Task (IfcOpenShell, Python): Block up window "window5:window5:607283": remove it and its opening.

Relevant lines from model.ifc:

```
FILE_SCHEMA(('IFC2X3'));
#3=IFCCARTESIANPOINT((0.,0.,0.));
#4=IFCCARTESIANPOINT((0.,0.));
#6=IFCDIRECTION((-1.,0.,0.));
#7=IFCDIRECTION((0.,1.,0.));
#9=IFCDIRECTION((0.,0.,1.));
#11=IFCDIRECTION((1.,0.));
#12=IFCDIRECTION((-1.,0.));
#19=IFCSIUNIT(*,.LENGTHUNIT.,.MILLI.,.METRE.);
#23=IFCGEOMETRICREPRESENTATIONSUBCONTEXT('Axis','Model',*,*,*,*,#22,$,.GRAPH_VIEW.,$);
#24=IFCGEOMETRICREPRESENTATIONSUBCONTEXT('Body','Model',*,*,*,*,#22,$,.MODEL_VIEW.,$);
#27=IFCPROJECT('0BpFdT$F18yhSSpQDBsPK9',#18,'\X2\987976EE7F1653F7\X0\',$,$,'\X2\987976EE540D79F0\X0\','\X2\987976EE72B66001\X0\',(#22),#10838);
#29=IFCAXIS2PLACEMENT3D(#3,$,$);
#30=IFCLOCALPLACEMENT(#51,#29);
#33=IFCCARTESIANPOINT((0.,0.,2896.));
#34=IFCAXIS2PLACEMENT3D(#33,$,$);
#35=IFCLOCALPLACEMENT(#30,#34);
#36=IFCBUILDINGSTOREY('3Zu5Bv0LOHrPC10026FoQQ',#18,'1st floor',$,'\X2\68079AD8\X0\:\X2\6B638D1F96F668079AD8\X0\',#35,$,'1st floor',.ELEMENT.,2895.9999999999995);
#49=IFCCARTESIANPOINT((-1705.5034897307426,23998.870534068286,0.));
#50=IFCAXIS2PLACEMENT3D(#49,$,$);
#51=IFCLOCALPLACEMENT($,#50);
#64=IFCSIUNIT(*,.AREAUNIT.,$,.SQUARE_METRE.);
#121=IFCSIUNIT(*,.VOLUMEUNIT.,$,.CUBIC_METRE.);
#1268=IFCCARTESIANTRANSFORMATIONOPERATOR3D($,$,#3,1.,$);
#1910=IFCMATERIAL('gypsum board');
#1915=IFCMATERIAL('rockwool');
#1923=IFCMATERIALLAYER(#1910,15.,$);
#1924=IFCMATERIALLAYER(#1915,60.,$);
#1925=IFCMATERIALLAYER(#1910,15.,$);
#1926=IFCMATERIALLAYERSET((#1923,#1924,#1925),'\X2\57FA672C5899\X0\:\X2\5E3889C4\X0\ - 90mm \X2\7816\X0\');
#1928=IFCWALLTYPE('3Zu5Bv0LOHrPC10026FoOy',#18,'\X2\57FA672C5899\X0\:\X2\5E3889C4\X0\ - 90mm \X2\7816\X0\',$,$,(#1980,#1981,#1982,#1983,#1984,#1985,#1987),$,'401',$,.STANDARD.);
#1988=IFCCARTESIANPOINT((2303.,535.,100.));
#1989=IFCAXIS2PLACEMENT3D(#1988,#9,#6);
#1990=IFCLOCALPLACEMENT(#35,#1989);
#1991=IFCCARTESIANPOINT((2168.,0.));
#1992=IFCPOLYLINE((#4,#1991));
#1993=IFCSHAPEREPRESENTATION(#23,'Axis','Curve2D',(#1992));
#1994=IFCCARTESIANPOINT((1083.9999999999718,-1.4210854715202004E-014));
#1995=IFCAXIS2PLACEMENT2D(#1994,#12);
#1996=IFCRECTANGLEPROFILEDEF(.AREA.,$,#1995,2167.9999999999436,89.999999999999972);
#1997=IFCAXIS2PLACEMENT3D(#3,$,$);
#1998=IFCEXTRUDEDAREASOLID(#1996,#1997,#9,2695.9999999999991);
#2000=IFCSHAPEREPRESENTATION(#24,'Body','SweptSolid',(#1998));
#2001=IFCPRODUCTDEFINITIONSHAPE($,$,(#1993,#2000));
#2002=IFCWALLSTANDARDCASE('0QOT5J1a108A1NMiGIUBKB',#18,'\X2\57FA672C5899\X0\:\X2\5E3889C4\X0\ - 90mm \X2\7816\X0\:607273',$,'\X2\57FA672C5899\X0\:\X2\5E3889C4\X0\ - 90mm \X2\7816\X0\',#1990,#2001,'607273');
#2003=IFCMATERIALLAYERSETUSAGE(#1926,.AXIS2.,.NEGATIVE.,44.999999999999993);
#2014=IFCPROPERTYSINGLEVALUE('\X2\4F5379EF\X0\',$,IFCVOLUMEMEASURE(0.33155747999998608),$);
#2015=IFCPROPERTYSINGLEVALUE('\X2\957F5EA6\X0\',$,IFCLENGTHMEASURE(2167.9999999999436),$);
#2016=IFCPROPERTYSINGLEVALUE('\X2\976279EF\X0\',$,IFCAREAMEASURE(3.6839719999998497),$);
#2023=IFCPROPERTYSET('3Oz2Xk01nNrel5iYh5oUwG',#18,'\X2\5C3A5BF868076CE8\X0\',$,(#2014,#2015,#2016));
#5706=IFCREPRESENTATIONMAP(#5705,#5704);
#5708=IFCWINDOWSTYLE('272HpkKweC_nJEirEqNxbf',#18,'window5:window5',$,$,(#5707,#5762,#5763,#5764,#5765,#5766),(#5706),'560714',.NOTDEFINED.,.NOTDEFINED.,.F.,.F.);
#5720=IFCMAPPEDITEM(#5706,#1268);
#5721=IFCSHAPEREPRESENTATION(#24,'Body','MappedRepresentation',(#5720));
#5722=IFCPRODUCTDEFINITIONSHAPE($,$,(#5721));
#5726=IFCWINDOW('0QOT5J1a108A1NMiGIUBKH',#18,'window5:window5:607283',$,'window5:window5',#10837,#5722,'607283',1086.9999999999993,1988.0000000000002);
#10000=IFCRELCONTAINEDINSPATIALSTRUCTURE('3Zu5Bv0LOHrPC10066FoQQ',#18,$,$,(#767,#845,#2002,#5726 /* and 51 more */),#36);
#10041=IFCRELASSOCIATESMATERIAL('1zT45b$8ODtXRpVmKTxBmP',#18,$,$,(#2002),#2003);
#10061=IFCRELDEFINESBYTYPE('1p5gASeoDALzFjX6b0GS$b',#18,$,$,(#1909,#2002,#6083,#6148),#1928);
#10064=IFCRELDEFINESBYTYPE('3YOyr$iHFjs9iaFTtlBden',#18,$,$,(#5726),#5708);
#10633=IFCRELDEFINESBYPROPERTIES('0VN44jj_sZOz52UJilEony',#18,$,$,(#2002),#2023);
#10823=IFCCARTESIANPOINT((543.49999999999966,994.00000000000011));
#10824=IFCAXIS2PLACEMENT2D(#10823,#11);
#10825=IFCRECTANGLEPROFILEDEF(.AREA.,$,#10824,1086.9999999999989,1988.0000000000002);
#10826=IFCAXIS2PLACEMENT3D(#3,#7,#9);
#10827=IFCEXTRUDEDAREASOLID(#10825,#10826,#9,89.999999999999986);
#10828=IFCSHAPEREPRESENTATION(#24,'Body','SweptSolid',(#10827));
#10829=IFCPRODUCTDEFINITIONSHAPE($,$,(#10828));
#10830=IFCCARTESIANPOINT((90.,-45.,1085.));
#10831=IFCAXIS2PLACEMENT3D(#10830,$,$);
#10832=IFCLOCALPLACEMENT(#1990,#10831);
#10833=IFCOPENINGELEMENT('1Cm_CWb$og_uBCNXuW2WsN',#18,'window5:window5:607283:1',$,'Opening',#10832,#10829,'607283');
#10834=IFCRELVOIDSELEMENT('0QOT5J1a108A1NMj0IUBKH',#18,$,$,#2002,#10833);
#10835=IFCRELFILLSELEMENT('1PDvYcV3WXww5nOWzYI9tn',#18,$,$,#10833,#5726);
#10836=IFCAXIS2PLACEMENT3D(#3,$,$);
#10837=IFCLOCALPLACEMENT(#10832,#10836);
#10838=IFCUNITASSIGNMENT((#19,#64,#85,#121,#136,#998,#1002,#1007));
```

```python
import ifcopenshell
import ifcopenshell.api.feature
import ifcopenshell.api.pset
import ifcopenshell.api.root
import ifcopenshell.geom
import ifcopenshell.util.element
import ifcopenshell.util.shape
import ifcopenshell.util.unit

model = ifcopenshell.open("model.ifc")
area_scale = ifcopenshell.util.unit.calculate_unit_scale(model, "AREAUNIT")
volume_scale = ifcopenshell.util.unit.calculate_unit_scale(model, "VOLUMEUNIT")
settings = ifcopenshell.geom.settings()


def volume(element):
    """Net volume in cubic metres, openings subtracted."""
    shape = ifcopenshell.geom.create_shape(settings, element)
    return ifcopenshell.util.shape.get_volume(shape.geometry)


window = model.by_guid("0QOT5J1a108A1NMiGIUBKH")
opening = window.FillsVoids[0].RelatingOpeningElement
wall = opening.VoidsElements[0].RelatingBuildingElement
before = volume(wall)

ifcopenshell.api.root.remove_product(model, product=window)
ifcopenshell.api.feature.remove_feature(model, feature=opening)

after = volume(wall)
thickness = 0.09  # wall thickness in metres

# Update the wall's stored quantities.
pset = model.by_id(ifcopenshell.util.element.get_pset(wall, "尺寸标注", should_inherit=False)["id"])
ifcopenshell.api.pset.edit_pset(model, pset=pset, properties={
    "体积": model.create_entity("IfcVolumeMeasure", after / volume_scale),
    "面积": model.create_entity("IfcAreaMeasure", after / thickness / area_scale),
})

print(f"wall volume {before:.3f} -> {after:.3f} m3")

model.write("model_updated.ifc")
```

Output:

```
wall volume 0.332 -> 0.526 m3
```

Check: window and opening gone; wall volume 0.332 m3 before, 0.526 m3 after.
